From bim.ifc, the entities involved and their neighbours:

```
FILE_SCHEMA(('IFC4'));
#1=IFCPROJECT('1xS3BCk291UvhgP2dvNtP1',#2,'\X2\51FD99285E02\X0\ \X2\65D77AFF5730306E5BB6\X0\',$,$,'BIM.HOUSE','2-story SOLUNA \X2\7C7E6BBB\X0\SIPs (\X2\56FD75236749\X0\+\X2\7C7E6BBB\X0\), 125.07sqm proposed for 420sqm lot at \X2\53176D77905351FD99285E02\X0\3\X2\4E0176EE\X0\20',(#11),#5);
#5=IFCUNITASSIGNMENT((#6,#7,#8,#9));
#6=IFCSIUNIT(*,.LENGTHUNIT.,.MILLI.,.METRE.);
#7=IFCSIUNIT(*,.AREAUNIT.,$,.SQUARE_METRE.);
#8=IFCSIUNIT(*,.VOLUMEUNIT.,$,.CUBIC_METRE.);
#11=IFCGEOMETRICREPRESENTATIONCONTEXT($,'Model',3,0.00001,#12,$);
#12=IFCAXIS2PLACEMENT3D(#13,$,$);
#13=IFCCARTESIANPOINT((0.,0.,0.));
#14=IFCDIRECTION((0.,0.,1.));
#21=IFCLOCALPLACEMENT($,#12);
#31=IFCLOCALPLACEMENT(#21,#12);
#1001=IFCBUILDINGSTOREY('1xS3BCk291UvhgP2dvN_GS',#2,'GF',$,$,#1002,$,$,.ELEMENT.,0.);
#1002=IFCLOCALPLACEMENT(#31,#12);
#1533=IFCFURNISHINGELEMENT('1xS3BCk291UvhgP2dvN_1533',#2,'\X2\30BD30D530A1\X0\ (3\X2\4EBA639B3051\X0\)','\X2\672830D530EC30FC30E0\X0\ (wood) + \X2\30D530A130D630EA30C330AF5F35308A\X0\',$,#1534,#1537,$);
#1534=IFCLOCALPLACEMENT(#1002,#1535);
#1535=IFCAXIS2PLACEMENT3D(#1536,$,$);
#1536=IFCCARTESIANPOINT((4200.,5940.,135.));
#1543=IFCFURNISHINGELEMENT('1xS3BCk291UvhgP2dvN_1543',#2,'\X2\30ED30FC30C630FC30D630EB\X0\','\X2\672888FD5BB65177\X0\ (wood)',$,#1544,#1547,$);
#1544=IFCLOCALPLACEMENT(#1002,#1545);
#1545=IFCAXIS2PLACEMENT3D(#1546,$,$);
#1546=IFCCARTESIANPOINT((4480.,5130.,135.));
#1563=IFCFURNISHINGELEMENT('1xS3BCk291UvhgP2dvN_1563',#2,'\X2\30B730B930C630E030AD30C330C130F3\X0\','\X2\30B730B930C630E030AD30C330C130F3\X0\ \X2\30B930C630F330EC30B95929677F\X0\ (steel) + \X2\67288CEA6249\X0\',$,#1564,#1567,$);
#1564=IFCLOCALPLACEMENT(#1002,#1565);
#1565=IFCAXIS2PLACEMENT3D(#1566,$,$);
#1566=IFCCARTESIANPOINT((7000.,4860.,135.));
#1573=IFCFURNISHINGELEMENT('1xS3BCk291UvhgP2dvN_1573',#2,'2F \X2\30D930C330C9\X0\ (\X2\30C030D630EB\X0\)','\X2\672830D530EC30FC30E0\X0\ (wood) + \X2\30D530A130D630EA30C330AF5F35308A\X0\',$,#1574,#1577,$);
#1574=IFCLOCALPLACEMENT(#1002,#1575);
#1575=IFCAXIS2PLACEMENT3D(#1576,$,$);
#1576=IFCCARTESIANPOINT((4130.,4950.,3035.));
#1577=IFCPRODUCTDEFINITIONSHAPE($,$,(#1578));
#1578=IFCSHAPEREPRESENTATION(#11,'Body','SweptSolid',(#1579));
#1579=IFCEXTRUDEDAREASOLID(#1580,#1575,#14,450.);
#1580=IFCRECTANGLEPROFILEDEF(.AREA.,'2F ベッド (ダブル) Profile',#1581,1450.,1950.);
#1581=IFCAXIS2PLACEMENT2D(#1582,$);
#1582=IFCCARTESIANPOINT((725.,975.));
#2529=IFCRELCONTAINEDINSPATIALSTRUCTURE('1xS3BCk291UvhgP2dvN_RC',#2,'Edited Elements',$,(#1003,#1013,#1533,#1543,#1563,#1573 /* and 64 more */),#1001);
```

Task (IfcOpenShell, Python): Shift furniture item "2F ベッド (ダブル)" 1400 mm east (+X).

```python
import ifcopenshell
import ifcopenshell.api.geometry
import ifcopenshell.util.placement

model = ifcopenshell.open("bim.ifc")

item = model.by_id(1573)
matrix = ifcopenshell.util.placement.get_local_placement(item.ObjectPlacement)
matrix[0, 3] += 1400.0
ifcopenshell.api.geometry.edit_object_placement(model, product=item, matrix=matrix, is_si=False)

print(ifcopenshell.util.placement.get_local_placement(item.ObjectPlacement).round(3) + 0.0)

model.write("bim_updated.ifc")
```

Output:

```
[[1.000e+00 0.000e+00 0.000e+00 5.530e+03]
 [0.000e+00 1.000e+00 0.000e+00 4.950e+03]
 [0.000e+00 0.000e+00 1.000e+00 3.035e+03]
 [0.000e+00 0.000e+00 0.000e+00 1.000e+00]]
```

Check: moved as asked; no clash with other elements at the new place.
